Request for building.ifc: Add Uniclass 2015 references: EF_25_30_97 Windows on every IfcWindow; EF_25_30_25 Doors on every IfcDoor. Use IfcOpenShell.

First a look at what the model holds.

```python
import ifcopenshell

model = ifcopenshell.open("building.ifc")
print(model.schema)
print("classifications:", [c.Name for c in model.by_type("IfcClassification")])
for ifc_class in ("IfcDoor", "IfcRoof", "IfcStair", "IfcWall", "IfcWindow"):
    print(ifc_class, len(model.by_type(ifc_class)))
```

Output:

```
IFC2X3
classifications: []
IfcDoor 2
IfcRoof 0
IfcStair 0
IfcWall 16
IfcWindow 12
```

```python
import ifcopenshell
import ifcopenshell.api.classification

model = ifcopenshell.open("building.ifc")

# IFC2X3 requires Source and Edition and has no link from the project to the system.
system = model.create_entity("IfcClassification", Source="NBS", Edition="2015", Name="Uniclass 2015")

codes = {
    "IfcWindow": ("EF_25_30_97", "Windows"),
    "IfcDoor": ("EF_25_30_25", "Doors"),
}
for ifc_class, (code, name) in codes.items():
    products = model.by_type(ifc_class)
    ifcopenshell.api.classification.add_reference(
        model, products=products, classification=system, identification=code, name=name
    )
    print(code, len(products))

model.write("building_updated.ifc")
```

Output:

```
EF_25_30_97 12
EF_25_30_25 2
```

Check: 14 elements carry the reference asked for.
